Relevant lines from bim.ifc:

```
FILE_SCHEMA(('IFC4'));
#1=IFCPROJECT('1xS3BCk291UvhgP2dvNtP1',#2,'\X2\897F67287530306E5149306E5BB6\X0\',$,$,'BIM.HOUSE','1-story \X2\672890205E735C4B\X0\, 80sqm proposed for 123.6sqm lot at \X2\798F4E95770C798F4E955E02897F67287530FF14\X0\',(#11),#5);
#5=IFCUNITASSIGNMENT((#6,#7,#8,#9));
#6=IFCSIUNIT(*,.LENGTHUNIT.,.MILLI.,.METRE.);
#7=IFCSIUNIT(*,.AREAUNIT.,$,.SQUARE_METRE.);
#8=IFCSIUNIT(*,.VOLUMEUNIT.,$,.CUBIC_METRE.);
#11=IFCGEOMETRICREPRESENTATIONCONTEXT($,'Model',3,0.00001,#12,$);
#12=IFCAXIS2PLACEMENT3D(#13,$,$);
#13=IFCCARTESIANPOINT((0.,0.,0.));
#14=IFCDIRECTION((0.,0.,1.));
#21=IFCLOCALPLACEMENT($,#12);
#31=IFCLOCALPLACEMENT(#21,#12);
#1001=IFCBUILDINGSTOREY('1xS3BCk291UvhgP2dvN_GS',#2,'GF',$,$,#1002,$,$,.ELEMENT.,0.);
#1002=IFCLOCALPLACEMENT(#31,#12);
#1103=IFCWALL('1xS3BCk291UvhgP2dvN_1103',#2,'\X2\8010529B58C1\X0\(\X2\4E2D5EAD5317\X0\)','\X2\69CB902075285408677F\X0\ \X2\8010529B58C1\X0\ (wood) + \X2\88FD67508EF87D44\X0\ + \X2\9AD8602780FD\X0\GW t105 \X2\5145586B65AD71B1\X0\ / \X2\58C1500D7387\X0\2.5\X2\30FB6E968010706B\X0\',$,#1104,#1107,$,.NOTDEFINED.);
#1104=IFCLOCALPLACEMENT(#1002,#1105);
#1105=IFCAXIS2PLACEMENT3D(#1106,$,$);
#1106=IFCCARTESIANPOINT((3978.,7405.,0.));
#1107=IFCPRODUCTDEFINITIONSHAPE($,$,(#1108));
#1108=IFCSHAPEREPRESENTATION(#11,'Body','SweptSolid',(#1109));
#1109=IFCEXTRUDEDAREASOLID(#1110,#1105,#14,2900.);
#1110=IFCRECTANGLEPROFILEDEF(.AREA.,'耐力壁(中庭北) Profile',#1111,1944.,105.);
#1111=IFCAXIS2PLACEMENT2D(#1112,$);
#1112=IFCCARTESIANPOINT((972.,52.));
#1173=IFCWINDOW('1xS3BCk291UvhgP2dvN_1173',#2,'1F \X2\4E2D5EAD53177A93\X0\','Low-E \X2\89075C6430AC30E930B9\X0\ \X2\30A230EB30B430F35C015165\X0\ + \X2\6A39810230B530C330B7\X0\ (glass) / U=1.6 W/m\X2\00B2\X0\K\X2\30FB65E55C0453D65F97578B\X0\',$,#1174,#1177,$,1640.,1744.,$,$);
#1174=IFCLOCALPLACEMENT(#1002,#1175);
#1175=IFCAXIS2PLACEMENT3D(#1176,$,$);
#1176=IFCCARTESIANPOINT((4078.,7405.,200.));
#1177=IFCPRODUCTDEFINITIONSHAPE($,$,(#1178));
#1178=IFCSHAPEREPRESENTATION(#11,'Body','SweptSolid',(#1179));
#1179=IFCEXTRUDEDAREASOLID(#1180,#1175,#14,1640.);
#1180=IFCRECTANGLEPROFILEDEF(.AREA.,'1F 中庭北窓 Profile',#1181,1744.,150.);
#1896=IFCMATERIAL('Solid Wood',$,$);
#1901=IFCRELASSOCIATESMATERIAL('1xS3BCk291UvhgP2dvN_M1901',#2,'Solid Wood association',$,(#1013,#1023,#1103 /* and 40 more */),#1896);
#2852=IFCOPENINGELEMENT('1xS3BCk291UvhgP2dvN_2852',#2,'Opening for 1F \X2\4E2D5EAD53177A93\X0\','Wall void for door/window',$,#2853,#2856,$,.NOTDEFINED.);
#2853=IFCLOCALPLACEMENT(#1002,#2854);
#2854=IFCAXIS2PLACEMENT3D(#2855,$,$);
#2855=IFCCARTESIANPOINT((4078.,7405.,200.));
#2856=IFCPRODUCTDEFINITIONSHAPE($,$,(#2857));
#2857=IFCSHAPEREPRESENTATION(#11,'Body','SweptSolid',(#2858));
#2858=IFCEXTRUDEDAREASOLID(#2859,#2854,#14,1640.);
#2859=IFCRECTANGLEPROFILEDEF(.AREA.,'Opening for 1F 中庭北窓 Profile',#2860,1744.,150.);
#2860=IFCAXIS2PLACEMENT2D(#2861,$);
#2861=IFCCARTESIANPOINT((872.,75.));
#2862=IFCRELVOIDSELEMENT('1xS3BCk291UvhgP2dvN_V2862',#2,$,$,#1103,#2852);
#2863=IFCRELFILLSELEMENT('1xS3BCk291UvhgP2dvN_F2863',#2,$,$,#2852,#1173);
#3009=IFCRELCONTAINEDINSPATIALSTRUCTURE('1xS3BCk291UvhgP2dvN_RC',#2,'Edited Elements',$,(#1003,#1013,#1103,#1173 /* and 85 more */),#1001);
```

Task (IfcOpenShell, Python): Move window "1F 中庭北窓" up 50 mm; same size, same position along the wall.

```python
import numpy as np
import ifcopenshell
import ifcopenshell.api.geometry
import ifcopenshell.util.placement
import ifcopenshell.util.unit

model = ifcopenshell.open("bim.ifc")
unit_scale = ifcopenshell.util.unit.calculate_unit_scale(model)

window = model.by_id(1173)
opening = window.FillsVoids[0].RelatingOpeningElement
dz = 50.0

shift = np.array([0.0, 0.0, dz])
# The window is not placed relative to its opening, so move both.
for product in (opening, window):
    matrix = ifcopenshell.util.placement.get_local_placement(product.ObjectPlacement)
    matrix[:3, 3] += shift
    ifcopenshell.api.geometry.edit_object_placement(model, product=product, matrix=matrix, is_si=False)

print(f"moved by {dz * unit_scale:+.3f} m")

model.write("bim_edited.ifc")
```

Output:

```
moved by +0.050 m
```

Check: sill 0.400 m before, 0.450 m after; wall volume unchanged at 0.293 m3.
